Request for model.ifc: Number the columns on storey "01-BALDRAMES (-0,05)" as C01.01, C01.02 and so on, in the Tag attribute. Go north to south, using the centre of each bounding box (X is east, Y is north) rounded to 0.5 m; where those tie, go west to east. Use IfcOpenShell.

First a look at what the model holds.

```python
import ifcopenshell
import ifcopenshell.util.element
import ifcopenshell.util.placement

model = ifcopenshell.open("model.ifc")
print(model.schema)
storey = next(s for s in model.by_type("IfcBuildingStorey") if s.Name == "01-BALDRAMES (-0,05)")
columns = [e for e in ifcopenshell.util.element.get_decomposition(storey) if e.is_a("IfcColumn")]
for e in sorted(columns, key=lambda e: e.id()):
    origin = ifcopenshell.util.placement.get_local_placement(e.ObjectPlacement)[:3, 3]
    print(e.id(), e.Tag, e.Name, origin.round(2) + 0.0, sep=" | ")
```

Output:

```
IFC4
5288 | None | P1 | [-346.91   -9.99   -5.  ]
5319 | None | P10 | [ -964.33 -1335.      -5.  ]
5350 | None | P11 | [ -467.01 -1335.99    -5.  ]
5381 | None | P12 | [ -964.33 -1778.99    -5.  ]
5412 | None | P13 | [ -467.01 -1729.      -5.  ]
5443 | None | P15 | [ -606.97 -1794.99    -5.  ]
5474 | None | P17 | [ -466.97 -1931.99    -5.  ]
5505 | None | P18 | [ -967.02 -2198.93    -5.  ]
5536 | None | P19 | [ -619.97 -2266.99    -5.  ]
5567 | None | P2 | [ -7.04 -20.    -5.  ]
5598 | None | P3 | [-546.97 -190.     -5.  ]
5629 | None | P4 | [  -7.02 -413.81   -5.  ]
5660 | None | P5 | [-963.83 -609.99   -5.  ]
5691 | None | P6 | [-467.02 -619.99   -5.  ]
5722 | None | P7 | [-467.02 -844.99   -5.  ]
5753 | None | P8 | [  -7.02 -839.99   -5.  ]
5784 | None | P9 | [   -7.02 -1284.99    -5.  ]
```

```python
import ifcopenshell
import ifcopenshell.geom
import ifcopenshell.util.element
import ifcopenshell.util.shape

model = ifcopenshell.open("model.ifc")
settings = ifcopenshell.geom.settings()
settings.set("use-world-coords", True)


def centre(element):
    shape = ifcopenshell.geom.create_shape(settings, element)
    return ifcopenshell.util.shape.get_bbox_centroid(shape.geometry)


storey = next(s for s in model.by_type("IfcBuildingStorey") if s.Name == "01-BALDRAMES (-0,05)")
columns = [e for e in ifcopenshell.util.element.get_decomposition(storey) if e.is_a("IfcColumn")]

# Insertion points can sit at a corner or the storey origin, so sort by the geometry (in metres).
centres = {e: centre(e) for e in columns}
columns.sort(key=lambda e: (-round(centres[e][1] / 0.5), centres[e][0]))

for i, e in enumerate(columns, start=1):
    number = f"C01.{i:02d}"
    e.Tag = number
    print(e.id(), number)

model.write("model-out.ifc")
```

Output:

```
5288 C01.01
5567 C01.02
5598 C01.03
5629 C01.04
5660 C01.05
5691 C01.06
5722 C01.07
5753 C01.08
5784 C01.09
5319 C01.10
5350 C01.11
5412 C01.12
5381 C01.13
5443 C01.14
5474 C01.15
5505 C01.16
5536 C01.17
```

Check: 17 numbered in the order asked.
